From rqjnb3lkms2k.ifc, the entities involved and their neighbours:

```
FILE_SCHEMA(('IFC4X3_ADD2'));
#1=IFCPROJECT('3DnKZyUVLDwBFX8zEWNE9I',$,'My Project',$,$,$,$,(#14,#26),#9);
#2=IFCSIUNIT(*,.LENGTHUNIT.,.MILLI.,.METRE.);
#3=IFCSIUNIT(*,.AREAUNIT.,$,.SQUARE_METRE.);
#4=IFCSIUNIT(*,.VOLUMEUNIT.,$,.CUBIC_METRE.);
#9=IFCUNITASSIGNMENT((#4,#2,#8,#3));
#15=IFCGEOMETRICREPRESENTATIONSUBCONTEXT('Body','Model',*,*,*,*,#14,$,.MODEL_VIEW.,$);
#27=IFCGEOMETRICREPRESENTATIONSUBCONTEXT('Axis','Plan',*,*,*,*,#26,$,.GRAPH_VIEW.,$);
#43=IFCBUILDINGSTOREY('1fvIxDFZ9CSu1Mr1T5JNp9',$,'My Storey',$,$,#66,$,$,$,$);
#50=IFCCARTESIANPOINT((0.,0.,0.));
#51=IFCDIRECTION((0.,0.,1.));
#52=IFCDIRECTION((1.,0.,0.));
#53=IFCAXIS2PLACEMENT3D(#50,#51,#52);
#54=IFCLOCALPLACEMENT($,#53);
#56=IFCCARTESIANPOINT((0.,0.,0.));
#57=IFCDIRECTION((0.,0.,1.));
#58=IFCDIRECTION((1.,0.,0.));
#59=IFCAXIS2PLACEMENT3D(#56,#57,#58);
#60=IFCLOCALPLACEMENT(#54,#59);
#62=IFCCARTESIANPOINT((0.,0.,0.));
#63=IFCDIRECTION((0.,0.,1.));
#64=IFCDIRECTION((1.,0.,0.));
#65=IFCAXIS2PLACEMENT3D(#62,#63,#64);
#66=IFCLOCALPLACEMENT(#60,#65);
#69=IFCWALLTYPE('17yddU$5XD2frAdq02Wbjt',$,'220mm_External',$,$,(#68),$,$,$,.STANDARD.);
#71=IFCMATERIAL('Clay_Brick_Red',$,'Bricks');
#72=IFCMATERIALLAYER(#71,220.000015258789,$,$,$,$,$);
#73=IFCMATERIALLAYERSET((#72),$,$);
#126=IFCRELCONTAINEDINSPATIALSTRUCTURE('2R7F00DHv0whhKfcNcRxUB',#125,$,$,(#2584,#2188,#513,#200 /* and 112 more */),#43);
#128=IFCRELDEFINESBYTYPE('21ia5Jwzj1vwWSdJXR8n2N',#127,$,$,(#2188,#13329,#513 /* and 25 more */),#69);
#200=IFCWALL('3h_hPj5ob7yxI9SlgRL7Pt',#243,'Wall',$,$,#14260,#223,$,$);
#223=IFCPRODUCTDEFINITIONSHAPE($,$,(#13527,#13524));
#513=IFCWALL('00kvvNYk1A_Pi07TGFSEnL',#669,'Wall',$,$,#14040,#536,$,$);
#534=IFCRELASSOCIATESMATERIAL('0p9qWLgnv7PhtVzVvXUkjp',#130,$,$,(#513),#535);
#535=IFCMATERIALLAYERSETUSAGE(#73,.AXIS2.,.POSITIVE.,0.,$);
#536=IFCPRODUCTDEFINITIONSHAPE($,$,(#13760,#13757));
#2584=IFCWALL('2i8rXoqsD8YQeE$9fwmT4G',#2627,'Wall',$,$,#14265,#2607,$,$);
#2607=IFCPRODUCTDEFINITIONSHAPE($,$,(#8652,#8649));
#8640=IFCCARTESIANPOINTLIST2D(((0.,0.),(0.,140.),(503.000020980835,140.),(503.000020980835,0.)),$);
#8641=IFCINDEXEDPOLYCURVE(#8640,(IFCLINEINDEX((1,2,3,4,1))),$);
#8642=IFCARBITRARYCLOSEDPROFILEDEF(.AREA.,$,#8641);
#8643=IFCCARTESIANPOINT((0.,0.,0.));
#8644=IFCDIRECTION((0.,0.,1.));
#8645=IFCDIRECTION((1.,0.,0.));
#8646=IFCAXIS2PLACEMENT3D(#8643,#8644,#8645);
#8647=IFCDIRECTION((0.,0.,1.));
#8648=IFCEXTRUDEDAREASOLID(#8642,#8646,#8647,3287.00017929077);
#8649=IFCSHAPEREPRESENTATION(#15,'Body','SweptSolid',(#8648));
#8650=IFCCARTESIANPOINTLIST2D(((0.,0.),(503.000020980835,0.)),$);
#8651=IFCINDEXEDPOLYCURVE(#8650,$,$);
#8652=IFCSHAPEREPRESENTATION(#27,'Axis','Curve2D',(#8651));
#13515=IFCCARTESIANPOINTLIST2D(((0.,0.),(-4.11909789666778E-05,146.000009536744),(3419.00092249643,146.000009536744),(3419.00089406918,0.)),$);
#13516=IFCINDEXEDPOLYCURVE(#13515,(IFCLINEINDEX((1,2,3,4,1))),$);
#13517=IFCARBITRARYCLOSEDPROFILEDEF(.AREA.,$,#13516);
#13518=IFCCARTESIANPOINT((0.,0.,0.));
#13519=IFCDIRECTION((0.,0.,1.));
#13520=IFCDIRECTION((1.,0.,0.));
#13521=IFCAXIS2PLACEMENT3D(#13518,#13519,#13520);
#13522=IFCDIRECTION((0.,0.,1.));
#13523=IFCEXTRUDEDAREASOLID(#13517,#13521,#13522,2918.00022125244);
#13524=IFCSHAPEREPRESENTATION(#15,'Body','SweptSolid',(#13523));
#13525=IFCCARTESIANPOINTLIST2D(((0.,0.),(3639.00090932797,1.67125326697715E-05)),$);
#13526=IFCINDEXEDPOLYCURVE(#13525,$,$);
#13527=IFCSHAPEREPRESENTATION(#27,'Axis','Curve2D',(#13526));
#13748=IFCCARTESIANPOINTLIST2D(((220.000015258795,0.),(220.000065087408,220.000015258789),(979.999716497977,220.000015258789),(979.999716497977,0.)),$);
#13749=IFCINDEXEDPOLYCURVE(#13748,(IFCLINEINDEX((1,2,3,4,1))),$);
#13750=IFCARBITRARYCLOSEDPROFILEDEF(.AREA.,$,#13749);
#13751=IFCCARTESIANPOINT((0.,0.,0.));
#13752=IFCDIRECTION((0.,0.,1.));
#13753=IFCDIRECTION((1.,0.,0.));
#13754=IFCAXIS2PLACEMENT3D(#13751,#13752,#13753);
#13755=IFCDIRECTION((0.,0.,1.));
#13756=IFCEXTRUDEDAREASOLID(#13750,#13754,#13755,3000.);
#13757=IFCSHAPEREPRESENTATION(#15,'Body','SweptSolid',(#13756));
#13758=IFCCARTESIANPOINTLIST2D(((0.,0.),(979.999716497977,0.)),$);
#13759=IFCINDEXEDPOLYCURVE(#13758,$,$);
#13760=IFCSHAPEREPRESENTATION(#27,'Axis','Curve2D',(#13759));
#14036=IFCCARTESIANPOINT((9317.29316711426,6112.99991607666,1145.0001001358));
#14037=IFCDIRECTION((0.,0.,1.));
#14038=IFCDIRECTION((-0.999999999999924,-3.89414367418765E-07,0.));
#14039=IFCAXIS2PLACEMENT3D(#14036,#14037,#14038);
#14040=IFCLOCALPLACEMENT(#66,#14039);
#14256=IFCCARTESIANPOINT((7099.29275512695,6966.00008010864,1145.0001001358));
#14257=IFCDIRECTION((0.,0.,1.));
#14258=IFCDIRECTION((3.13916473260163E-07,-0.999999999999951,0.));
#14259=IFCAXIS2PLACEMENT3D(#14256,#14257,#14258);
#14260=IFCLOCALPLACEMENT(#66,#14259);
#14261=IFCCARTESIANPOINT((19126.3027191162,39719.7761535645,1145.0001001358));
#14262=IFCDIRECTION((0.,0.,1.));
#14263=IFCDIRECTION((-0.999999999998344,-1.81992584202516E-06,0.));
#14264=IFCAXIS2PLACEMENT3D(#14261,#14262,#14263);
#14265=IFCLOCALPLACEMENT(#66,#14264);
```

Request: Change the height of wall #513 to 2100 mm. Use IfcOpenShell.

```python
import ifcopenshell
import ifcopenshell.geom
import ifcopenshell.util.representation
import ifcopenshell.util.shape
import ifcopenshell.util.unit

model = ifcopenshell.open("rqjnb3lkms2k.ifc")
unit_scale = ifcopenshell.util.unit.calculate_unit_scale(model)
settings = ifcopenshell.geom.settings()


def volume(element):
    """Net volume in cubic metres, openings subtracted."""
    shape = ifcopenshell.geom.create_shape(settings, element)
    return ifcopenshell.util.shape.get_volume(shape.geometry)


wall = model.by_id(513)
before = volume(wall)

body = ifcopenshell.util.representation.get_representation(wall, "Model", "Body")
solid = body.Items[0]
old_height = solid.Depth
solid.Depth = 2.1 / unit_scale
after = volume(wall)

print(f"height {old_height:g} -> {solid.Depth:g}, volume {before:.3f} -> {after:.3f} m3")

model.write("rqjnb3lkms2k-out.ifc")
```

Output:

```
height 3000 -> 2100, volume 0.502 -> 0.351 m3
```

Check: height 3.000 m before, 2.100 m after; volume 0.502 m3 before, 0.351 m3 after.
